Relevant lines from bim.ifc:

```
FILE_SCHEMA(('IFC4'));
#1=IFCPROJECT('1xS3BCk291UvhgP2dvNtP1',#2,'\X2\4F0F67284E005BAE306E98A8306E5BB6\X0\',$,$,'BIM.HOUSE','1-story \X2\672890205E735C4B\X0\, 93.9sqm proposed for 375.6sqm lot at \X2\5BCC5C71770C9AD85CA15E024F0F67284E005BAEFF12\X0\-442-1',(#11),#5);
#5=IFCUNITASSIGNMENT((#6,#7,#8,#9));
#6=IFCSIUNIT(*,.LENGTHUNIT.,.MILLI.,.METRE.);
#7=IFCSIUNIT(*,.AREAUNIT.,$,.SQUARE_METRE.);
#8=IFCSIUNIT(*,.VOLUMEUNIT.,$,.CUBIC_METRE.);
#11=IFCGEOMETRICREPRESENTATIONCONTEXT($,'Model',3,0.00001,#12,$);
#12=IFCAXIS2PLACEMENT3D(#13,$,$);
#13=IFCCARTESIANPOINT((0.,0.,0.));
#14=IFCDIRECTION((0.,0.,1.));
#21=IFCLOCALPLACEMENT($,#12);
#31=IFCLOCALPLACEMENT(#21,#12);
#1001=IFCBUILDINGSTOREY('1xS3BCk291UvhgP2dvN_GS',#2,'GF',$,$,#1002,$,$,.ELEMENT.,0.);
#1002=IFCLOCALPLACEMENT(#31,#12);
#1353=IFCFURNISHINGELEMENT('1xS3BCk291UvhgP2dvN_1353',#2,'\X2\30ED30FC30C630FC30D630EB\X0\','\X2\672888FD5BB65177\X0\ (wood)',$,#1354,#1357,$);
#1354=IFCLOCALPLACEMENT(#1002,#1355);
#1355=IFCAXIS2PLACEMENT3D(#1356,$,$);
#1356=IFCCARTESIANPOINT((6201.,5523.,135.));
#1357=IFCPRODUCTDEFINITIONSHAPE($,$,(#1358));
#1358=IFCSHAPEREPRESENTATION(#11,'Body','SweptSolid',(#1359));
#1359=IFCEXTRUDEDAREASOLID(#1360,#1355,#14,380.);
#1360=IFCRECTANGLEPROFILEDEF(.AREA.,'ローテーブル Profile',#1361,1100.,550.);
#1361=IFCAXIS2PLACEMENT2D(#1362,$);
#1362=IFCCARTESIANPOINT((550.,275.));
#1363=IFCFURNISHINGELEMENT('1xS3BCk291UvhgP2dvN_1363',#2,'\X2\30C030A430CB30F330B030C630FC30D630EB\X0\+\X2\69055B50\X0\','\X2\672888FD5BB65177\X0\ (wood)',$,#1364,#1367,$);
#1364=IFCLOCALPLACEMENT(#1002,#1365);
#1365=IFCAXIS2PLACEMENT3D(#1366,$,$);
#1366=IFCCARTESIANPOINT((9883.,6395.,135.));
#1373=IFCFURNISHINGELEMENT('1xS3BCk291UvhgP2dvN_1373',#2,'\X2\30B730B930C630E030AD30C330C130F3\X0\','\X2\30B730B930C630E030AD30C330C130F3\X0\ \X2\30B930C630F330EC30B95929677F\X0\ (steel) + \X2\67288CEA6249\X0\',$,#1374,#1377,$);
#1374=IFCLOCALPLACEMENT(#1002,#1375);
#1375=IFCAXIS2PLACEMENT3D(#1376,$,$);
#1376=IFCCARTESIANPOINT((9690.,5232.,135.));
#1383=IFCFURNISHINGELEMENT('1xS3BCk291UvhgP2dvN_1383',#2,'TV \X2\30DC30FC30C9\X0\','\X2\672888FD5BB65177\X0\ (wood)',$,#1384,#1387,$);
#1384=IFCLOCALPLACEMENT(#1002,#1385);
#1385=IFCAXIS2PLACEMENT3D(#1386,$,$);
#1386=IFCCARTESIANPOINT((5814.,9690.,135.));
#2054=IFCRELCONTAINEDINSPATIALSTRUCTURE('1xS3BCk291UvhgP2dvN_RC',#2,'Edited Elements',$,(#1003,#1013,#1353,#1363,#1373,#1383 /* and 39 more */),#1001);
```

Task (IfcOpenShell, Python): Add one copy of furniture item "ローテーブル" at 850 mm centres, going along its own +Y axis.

```python
import ifcopenshell
import ifcopenshell.api.geometry
import ifcopenshell.api.root
import ifcopenshell.util.element
import ifcopenshell.util.placement
import ifcopenshell.util.unit

model = ifcopenshell.open("bim.ifc")
unit_scale = ifcopenshell.util.unit.calculate_unit_scale(model)


def reuse_history(source, copy):
    """copy_class also copies each property set's owner history, people and application; keep the originals."""
    for rel in copy.IsDefinedBy:
        if rel.is_a("IfcRelDefinesByProperties") and (history := rel.RelatingPropertyDefinition.OwnerHistory):
            rel.RelatingPropertyDefinition.OwnerHistory = source.OwnerHistory
            ifcopenshell.util.element.remove_deep2(model, history)


source = model.by_id(1353)
base = ifcopenshell.util.placement.get_local_placement(source.ObjectPlacement)
step = base[:3, 1] * 0.85 / unit_scale

for i in range(1, 2):
    copy = ifcopenshell.api.root.copy_class(model, product=source)
    copy.Representation = ifcopenshell.util.element.copy_deep(
        model, source.Representation, exclude=["IfcGeometricRepresentationContext", "IfcRepresentationMap"]
    )
    reuse_history(source, copy)
    matrix = base.copy()
    matrix[:3, 3] += i * step
    print("added at", matrix[:3, 3].round(3) + 0.0)
    ifcopenshell.api.geometry.edit_object_placement(model, product=copy, matrix=matrix, is_si=False)

model.write("bim-out.ifc")
```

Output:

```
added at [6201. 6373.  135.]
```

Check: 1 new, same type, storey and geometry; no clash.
